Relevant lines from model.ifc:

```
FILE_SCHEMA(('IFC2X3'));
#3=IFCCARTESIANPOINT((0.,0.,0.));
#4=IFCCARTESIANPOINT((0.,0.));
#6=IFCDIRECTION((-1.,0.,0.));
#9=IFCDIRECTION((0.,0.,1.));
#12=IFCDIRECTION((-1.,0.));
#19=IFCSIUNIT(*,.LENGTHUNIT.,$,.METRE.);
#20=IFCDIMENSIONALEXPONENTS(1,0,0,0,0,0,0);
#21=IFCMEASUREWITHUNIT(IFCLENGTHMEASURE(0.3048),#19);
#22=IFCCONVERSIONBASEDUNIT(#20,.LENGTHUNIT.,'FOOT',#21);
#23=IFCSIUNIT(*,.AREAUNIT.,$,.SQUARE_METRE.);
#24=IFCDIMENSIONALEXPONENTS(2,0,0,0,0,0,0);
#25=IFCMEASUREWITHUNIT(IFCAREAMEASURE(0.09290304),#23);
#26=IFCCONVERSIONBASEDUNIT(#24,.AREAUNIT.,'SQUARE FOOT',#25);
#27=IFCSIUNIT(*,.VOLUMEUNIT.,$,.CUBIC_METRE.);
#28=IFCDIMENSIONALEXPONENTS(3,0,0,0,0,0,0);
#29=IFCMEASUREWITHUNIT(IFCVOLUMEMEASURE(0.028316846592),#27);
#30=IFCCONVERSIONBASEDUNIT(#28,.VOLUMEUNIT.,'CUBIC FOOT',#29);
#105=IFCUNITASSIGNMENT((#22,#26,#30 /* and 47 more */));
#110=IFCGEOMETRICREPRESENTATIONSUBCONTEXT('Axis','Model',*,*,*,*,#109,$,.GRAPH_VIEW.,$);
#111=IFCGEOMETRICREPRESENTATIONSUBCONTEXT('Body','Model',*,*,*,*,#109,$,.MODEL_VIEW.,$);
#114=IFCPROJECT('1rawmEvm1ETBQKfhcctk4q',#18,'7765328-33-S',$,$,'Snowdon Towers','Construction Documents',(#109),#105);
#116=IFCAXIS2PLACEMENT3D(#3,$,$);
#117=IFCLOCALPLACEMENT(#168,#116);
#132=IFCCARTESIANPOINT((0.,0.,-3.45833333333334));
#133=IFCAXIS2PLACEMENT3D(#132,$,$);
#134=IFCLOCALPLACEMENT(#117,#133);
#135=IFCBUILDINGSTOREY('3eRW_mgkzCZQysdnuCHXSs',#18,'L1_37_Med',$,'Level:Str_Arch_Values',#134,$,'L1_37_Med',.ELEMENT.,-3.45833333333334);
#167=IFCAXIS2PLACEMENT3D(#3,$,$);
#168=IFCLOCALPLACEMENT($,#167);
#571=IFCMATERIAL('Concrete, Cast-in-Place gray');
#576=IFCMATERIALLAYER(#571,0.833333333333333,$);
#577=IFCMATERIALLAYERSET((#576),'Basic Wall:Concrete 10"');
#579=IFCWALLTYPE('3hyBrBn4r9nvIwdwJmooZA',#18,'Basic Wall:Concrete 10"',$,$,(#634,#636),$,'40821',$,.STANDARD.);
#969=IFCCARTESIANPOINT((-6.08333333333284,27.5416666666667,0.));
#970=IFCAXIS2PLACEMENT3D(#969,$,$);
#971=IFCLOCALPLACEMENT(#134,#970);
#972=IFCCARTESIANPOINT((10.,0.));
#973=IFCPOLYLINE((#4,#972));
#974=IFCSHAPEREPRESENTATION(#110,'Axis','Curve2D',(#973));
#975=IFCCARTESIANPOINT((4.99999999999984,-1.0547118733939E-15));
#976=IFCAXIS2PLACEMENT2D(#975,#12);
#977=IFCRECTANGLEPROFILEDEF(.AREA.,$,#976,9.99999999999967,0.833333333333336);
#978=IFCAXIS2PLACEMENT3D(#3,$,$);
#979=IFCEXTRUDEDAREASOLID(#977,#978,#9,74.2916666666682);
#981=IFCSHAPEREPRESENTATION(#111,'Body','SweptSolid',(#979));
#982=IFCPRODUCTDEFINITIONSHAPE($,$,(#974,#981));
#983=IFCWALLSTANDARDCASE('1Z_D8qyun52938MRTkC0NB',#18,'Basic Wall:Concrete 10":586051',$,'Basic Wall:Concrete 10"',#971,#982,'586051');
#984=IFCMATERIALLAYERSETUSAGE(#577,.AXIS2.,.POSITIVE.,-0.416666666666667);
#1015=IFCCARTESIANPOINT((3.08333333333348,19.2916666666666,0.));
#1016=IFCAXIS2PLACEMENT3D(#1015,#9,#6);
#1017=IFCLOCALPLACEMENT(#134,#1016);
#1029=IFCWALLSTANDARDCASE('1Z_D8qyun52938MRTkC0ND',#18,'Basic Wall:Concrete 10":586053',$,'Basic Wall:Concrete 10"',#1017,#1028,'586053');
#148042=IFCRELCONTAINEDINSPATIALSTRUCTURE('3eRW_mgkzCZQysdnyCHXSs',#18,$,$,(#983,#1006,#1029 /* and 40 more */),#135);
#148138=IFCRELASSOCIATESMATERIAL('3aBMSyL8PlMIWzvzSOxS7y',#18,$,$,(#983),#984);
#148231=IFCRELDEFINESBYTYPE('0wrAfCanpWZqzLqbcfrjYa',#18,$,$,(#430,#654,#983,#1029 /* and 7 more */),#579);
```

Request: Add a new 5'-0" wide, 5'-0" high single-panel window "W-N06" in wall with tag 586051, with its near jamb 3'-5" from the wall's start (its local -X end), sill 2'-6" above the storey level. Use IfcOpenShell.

```python
import numpy as np
import ifcopenshell
import ifcopenshell.api.feature
import ifcopenshell.api.geometry
import ifcopenshell.api.root
import ifcopenshell.api.spatial
import ifcopenshell.api.type
import ifcopenshell.geom
import ifcopenshell.util.element
import ifcopenshell.util.placement
import ifcopenshell.util.representation
import ifcopenshell.util.shape
import ifcopenshell.util.unit

model = ifcopenshell.open("model.ifc")
unit_scale = ifcopenshell.util.unit.calculate_unit_scale(model)
settings = ifcopenshell.geom.settings()


def volume(element):
    """Net volume in cubic metres, openings subtracted."""
    shape = ifcopenshell.geom.create_shape(settings, element)
    return ifcopenshell.util.shape.get_volume(shape.geometry)


wall = model.by_id(983)
storey = ifcopenshell.util.element.get_container(wall, ifc_class="IfcBuildingStorey")
context = ifcopenshell.util.representation.get_context(model, "Model", "Body", "MODEL_VIEW")
before = volume(wall)

width, height, from_end, sill = 1.524, 1.524, 1.0414, 0.762  # metres

# The wall runs along its own X axis, and the end named is its -X end.
wall_shape = ifcopenshell.geom.create_shape(settings, wall)
x, y, z = ifcopenshell.util.shape.get_vertices(wall_shape.geometry).T
start = x.min() + from_end
face, thickness = float(y.min()), float(y.max() - y.min())
wall_matrix = ifcopenshell.util.placement.get_local_placement(wall.ObjectPlacement)
level = ifcopenshell.util.placement.get_local_placement(storey.ObjectPlacement)[2, 3]


def in_wall(x, y):
    """Placement at x, y metres in the wall's axes, at sill height."""
    matrix = wall_matrix.copy()
    matrix[:, 3] = wall_matrix @ np.array([x / unit_scale, y / unit_scale, 0.0, 1.0])
    matrix[2, 3] = level + sill / unit_scale
    return matrix


# Opening: a box that overshoots both wall faces by 50 mm.
opening = ifcopenshell.api.root.create_entity(model, ifc_class="IfcOpeningElement")
box = ifcopenshell.api.geometry.add_wall_representation(
    model, context=context, length=width, height=height, thickness=thickness + 0.1
)
ifcopenshell.api.geometry.assign_representation(model, product=opening, representation=box)
ifcopenshell.api.geometry.edit_object_placement(model, product=opening, matrix=in_wall(start, face - 0.05), is_si=False)
ifcopenshell.api.feature.add_feature(model, feature=opening, element=wall)

window = ifcopenshell.api.root.create_entity(model, ifc_class="IfcWindow", name="W-N06")
window.OverallWidth, window.OverallHeight = width / unit_scale, height / unit_scale
body = ifcopenshell.api.geometry.add_window_representation(
    model,
    context=context,
    overall_width=window.OverallWidth,
    overall_height=window.OverallHeight,
    partition_type="SINGLE_PANEL",
)
ifcopenshell.api.geometry.assign_representation(model, product=window, representation=body)
ifcopenshell.api.spatial.assign_container(model, products=[window], relating_structure=storey)
fills = ifcopenshell.api.feature.add_filling(model, opening=opening, element=window)
fills.OwnerHistory = window.OwnerHistory  # required in IFC2X3

# IFC2X3 keeps the operation on the window style.
style = ifcopenshell.api.root.create_entity(model, ifc_class="IfcWindowStyle", name="W-N06")
style.OperationType, style.ConstructionType = "SINGLE_PANEL", "NOTDEFINED"
style.ParameterTakesPrecedence = style.Sizeable = False
ifcopenshell.api.type.assign_type(model, related_objects=[window], relating_type=style)

# Centre the window in the wall's thickness.
ifcopenshell.api.geometry.edit_object_placement(model, product=window, matrix=in_wall(start, face), is_si=False)
window_shape = ifcopenshell.geom.create_shape(settings, window)
depth = ifcopenshell.util.shape.get_vertices(window_shape.geometry)[:, 1]
offset = face + thickness / 2 - (depth.min() + depth.max()) / 2
ifcopenshell.api.geometry.edit_object_placement(model, product=window, matrix=in_wall(start, offset), is_si=False)

after = volume(wall)

print(f"wall volume {before:.3f} -> {after:.3f} m3")

model.write("model_edited.ifc")
```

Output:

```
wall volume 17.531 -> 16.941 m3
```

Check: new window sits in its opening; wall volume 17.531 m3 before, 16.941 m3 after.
